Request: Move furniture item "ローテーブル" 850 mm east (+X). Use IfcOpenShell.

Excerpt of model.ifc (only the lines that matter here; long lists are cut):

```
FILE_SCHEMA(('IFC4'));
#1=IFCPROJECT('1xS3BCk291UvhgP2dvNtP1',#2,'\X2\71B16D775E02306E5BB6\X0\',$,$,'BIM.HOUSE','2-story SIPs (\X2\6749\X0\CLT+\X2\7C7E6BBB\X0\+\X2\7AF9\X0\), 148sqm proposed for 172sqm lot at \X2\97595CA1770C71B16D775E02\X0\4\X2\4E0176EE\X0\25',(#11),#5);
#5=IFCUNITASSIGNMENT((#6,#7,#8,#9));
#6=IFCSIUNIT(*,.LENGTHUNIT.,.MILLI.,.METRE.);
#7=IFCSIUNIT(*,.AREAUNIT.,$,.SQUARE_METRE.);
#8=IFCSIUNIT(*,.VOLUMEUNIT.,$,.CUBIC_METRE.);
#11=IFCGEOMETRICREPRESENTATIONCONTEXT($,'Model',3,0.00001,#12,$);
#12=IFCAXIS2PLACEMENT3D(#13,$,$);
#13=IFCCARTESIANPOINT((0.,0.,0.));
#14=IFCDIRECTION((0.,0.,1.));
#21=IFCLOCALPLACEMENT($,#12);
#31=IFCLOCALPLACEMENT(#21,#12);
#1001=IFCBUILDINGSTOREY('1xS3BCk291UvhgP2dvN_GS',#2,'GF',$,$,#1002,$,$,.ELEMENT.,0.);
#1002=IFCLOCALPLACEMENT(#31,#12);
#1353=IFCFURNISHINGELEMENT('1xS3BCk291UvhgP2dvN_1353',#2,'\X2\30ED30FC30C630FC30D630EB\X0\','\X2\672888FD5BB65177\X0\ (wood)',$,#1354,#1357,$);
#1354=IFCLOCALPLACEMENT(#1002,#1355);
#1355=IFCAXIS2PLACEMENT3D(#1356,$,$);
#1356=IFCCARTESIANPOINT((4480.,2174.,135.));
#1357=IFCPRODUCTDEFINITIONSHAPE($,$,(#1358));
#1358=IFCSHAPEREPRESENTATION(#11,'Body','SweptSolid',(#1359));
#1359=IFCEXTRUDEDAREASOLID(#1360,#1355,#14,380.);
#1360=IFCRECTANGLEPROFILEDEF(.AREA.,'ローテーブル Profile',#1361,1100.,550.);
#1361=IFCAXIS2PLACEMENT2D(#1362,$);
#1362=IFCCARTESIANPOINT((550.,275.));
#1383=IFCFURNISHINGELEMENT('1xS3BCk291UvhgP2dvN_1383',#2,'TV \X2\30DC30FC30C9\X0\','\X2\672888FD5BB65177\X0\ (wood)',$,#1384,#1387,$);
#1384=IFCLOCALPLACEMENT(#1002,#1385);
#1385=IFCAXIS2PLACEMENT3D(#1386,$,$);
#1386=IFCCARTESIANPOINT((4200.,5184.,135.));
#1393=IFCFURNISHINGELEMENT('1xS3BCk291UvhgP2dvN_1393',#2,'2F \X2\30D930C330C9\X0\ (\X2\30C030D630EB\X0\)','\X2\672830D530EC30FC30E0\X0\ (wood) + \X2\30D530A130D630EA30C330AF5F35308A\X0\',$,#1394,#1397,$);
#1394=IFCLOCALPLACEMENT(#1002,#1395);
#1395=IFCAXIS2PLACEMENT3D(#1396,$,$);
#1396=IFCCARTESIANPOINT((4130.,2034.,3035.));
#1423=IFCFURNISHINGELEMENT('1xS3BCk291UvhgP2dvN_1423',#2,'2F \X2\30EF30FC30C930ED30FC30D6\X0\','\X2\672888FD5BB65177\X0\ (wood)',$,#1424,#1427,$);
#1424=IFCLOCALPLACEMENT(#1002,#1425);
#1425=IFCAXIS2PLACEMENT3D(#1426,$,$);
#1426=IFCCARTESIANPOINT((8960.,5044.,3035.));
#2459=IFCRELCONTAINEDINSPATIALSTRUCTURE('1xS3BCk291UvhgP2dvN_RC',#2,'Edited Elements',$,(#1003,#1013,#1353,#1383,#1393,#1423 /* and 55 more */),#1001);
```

```python
import ifcopenshell
import ifcopenshell.api.geometry
import ifcopenshell.util.placement
import ifcopenshell.util.unit

model = ifcopenshell.open("model.ifc")
unit_scale = ifcopenshell.util.unit.calculate_unit_scale(model)

item = model.by_guid("1xS3BCk291UvhgP2dvN_1353")
matrix = ifcopenshell.util.placement.get_local_placement(item.ObjectPlacement)
matrix[0, 3] += 0.85 / unit_scale
ifcopenshell.api.geometry.edit_object_placement(model, product=item, matrix=matrix, is_si=False)

print(ifcopenshell.util.placement.get_local_placement(item.ObjectPlacement).round(3) + 0.0)

model.write("model_rev.ifc")
```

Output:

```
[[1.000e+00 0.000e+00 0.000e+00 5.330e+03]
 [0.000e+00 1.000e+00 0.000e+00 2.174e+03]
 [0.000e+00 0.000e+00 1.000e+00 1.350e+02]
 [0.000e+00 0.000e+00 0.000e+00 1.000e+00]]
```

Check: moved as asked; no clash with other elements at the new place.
